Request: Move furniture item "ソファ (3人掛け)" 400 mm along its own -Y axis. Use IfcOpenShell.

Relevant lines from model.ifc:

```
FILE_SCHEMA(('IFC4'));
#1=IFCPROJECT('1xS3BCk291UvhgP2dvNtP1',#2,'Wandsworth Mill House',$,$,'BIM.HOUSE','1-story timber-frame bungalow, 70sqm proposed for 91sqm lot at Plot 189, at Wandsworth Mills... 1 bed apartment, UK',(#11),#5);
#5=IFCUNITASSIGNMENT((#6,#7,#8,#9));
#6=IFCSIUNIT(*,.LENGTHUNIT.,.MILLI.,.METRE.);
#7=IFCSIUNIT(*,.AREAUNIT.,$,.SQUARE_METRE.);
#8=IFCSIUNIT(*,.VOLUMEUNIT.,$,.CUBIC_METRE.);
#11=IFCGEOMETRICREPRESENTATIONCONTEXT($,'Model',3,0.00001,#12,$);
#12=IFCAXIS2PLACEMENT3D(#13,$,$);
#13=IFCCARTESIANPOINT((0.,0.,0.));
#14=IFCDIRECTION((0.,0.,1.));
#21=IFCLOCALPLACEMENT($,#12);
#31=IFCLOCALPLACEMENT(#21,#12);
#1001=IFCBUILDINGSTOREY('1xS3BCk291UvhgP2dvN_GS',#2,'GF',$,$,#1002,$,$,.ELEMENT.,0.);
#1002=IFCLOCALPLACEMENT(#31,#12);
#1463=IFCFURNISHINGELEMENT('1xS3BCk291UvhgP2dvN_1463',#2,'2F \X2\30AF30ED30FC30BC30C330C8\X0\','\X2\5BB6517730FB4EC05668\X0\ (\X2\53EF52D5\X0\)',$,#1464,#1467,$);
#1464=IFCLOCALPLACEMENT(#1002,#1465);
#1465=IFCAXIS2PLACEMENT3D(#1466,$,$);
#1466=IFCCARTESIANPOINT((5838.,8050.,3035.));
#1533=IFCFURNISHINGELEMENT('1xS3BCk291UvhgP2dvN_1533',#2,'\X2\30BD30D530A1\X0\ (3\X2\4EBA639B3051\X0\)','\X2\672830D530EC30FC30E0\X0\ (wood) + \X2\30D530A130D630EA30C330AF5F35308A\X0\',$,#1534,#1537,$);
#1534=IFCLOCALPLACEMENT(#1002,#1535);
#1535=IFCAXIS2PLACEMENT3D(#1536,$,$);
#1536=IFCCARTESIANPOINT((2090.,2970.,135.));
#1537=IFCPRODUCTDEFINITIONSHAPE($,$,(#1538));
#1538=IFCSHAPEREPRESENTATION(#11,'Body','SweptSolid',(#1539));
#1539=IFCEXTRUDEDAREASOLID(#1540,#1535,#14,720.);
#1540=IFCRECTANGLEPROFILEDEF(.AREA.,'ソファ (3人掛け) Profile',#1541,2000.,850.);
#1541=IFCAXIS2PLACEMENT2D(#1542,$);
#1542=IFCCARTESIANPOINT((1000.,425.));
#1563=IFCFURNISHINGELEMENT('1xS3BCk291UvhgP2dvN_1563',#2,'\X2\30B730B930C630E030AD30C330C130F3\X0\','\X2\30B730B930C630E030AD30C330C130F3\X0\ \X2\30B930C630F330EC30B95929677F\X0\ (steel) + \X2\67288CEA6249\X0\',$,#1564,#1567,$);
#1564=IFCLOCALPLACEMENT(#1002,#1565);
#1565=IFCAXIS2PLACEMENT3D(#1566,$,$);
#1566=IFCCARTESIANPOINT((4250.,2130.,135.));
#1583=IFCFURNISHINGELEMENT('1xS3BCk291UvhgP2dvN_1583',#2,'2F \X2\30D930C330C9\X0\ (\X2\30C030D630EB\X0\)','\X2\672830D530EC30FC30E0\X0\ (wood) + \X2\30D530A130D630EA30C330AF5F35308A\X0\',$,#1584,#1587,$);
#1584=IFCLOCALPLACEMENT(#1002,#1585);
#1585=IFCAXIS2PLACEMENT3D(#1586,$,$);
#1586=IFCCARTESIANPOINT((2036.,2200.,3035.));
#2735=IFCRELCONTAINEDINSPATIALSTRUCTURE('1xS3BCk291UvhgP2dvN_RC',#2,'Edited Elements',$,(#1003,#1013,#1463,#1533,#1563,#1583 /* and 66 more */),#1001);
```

```python
import ifcopenshell
import ifcopenshell.api.geometry
import ifcopenshell.util.placement

model = ifcopenshell.open("model.ifc")

item = model.by_id(1533)
matrix = ifcopenshell.util.placement.get_local_placement(item.ObjectPlacement)
matrix[:3, 3] -= matrix[:3, 1] * 400.0
ifcopenshell.api.geometry.edit_object_placement(model, product=item, matrix=matrix, is_si=False)

print(ifcopenshell.util.placement.get_local_placement(item.ObjectPlacement).round(3) + 0.0)

model.write("model_edited.ifc")
```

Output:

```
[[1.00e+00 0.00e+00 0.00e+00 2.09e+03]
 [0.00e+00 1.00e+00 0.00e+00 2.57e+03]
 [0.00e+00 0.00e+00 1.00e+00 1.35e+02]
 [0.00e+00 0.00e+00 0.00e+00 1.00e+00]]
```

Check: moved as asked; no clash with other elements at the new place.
